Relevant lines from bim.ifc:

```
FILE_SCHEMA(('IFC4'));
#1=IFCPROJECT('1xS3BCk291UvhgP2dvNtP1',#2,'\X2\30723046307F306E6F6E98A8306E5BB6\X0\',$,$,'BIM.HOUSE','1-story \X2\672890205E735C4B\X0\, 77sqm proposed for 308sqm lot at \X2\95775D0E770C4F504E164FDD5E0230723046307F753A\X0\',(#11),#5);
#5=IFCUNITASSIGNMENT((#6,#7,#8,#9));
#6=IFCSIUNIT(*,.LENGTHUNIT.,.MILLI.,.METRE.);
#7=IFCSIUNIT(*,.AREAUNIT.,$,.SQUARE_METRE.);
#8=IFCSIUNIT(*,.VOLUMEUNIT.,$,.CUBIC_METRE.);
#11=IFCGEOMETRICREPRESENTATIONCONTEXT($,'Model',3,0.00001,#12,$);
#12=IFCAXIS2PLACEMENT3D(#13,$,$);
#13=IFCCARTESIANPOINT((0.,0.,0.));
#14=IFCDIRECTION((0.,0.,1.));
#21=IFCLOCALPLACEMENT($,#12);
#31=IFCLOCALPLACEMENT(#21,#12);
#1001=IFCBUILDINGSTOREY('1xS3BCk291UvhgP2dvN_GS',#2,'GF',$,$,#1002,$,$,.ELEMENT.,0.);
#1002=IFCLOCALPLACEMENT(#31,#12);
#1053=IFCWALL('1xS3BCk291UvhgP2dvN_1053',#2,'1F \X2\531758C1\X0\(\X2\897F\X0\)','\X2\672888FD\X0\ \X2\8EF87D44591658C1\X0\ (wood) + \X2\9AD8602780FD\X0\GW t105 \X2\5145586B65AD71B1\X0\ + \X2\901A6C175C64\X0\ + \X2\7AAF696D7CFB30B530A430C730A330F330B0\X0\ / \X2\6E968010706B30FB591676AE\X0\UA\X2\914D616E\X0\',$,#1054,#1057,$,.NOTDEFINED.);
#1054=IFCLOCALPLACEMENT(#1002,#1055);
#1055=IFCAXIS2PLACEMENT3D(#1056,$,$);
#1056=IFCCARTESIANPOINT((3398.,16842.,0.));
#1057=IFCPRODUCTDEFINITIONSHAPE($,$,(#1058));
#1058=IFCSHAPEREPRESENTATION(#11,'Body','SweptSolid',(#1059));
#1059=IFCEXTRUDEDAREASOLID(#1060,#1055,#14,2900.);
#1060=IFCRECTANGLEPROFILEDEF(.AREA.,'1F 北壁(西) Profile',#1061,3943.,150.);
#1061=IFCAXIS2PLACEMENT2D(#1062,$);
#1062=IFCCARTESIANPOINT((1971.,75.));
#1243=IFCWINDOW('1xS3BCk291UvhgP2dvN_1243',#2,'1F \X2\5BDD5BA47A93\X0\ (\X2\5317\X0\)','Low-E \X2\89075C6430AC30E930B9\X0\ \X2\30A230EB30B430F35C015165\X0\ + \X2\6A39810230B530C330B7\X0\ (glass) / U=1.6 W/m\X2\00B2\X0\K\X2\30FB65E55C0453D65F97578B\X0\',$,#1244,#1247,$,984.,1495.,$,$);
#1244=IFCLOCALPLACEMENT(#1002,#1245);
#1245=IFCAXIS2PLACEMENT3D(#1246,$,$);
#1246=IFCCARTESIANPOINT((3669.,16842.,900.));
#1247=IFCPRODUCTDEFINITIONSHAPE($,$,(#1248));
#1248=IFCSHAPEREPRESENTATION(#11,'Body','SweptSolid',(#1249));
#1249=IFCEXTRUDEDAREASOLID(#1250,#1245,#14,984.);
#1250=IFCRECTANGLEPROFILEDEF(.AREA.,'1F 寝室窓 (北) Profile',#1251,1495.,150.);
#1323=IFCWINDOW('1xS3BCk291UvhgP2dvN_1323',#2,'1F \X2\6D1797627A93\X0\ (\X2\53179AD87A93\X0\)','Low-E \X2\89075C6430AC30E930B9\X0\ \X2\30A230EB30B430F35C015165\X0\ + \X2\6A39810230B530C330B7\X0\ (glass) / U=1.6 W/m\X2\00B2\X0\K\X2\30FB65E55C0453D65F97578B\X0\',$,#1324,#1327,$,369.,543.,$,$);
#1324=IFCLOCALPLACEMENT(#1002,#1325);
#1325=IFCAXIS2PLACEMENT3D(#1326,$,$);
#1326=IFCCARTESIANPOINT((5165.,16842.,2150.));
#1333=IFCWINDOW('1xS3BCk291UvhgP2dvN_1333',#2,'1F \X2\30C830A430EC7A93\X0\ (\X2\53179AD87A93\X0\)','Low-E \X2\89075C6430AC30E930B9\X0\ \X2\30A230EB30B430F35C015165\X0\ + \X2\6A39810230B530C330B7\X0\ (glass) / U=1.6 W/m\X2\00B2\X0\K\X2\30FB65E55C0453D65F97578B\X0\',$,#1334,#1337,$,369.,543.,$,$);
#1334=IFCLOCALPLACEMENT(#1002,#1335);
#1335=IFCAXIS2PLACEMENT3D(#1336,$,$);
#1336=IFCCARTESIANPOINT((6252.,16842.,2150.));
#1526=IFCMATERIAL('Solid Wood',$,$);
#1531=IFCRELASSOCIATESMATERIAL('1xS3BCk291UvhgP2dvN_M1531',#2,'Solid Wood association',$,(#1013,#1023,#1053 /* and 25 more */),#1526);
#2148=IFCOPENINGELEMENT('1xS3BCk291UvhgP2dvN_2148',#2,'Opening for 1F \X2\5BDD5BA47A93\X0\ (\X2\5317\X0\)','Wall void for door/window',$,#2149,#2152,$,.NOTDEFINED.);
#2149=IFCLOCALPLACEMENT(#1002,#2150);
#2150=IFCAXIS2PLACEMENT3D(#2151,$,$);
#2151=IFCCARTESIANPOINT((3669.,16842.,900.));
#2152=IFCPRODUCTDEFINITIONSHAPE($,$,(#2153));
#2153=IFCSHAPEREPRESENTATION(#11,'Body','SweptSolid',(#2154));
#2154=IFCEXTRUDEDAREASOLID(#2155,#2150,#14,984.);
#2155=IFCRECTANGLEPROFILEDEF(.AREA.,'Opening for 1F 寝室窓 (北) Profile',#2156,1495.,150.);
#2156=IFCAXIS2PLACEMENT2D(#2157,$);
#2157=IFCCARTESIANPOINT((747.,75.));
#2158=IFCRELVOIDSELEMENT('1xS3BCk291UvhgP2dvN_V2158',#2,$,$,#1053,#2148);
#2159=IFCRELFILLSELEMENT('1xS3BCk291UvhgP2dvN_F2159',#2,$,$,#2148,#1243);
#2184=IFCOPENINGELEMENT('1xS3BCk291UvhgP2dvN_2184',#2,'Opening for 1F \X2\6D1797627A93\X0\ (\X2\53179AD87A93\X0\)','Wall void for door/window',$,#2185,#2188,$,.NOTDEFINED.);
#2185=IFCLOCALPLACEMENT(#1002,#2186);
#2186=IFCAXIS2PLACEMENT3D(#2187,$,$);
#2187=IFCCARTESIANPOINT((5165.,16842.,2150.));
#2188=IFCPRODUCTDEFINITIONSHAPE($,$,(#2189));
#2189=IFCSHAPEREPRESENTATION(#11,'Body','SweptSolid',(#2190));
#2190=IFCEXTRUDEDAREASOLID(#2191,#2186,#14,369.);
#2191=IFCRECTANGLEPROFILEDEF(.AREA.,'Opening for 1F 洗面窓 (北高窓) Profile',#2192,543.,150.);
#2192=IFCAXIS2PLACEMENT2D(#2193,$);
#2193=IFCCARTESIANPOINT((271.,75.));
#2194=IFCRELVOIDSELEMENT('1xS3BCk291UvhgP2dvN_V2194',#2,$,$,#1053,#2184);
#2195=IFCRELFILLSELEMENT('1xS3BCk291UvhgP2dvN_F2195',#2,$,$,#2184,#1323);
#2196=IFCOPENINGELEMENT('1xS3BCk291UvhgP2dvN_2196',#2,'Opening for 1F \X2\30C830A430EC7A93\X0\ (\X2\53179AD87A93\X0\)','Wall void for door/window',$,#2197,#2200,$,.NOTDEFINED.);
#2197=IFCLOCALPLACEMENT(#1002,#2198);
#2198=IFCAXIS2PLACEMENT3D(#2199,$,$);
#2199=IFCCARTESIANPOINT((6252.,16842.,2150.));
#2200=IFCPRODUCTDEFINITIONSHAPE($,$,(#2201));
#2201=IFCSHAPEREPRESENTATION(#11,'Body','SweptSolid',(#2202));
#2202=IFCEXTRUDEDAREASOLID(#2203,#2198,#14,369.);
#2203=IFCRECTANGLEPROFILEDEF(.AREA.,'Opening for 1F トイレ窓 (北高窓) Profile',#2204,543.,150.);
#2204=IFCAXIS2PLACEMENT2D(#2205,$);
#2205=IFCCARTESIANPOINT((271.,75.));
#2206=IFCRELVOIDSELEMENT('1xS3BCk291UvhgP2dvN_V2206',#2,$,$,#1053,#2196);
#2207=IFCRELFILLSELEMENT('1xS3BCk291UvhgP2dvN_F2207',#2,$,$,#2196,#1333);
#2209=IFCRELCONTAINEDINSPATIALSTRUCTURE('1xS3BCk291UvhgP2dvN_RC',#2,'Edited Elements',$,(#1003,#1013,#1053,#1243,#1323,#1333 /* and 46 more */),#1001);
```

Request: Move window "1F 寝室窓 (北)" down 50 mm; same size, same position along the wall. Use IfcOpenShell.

```python
import numpy as np
import ifcopenshell
import ifcopenshell.api.geometry
import ifcopenshell.util.placement
import ifcopenshell.util.unit

model = ifcopenshell.open("bim.ifc")
unit_scale = ifcopenshell.util.unit.calculate_unit_scale(model)

window = model.by_guid("1xS3BCk291UvhgP2dvN_1243")
opening = window.FillsVoids[0].RelatingOpeningElement
dz = -0.05 / unit_scale

shift = np.array([0.0, 0.0, dz])
# The window is not placed relative to its opening, so move both.
for product in (opening, window):
    matrix = ifcopenshell.util.placement.get_local_placement(product.ObjectPlacement)
    matrix[:3, 3] += shift
    ifcopenshell.api.geometry.edit_object_placement(model, product=product, matrix=matrix, is_si=False)

print(f"moved by {dz * unit_scale:+.3f} m")

model.write("bim_updated.ifc")
```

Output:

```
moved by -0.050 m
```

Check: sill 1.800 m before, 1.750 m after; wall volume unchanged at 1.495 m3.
